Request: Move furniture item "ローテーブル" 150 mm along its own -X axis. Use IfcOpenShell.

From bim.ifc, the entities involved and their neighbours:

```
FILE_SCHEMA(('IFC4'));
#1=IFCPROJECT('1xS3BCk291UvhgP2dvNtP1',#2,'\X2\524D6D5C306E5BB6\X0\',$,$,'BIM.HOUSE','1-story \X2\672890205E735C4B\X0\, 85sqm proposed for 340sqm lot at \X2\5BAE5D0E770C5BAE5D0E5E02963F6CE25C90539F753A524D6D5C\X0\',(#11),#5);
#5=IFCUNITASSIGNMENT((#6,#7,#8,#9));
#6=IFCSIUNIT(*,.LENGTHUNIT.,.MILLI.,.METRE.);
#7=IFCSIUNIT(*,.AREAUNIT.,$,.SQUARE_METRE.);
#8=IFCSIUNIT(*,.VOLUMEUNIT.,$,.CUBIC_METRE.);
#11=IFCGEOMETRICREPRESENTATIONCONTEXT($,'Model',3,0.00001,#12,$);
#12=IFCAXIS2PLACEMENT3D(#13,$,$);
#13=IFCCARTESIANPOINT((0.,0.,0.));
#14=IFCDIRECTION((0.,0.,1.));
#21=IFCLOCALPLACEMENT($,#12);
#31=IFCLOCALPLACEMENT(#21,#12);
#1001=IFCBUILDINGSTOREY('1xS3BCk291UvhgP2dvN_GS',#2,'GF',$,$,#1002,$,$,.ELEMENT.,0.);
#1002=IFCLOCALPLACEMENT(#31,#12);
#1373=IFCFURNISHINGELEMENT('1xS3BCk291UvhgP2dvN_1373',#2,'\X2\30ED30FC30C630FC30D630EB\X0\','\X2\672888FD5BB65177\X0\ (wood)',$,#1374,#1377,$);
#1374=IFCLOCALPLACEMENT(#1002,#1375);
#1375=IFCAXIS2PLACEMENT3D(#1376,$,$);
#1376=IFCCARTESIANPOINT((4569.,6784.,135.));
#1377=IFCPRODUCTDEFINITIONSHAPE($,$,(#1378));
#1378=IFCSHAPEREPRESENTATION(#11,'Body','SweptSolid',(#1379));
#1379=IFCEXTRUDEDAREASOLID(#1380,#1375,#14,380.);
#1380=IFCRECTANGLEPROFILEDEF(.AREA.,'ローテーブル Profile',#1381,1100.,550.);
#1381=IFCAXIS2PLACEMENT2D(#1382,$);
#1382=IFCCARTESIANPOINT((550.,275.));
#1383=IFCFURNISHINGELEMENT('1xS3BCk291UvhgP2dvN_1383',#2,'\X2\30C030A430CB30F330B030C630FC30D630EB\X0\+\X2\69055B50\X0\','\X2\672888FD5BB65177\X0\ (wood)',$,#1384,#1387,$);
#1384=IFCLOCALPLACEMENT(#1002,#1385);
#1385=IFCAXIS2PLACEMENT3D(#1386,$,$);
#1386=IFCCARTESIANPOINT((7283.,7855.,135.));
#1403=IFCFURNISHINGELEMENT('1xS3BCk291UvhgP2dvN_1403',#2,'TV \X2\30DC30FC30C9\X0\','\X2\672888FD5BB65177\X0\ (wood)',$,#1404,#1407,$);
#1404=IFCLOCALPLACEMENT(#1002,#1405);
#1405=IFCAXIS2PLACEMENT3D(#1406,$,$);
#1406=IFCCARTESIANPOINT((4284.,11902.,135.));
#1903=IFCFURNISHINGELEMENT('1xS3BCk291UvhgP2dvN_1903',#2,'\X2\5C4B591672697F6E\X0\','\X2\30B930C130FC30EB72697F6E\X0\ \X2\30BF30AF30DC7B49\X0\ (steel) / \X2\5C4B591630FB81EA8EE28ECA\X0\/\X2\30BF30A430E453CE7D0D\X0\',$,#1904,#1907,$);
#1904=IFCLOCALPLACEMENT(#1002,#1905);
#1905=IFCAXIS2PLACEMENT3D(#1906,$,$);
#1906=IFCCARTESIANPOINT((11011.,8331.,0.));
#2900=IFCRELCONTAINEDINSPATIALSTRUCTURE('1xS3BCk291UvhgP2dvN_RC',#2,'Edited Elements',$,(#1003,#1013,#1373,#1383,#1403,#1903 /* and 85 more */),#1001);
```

```python
import ifcopenshell
import ifcopenshell.api.geometry
import ifcopenshell.util.placement
import ifcopenshell.util.unit

model = ifcopenshell.open("bim.ifc")
unit_scale = ifcopenshell.util.unit.calculate_unit_scale(model)

item = model.by_guid("1xS3BCk291UvhgP2dvN_1373")
matrix = ifcopenshell.util.placement.get_local_placement(item.ObjectPlacement)
matrix[:3, 3] -= matrix[:3, 0] * 0.15 / unit_scale
ifcopenshell.api.geometry.edit_object_placement(model, product=item, matrix=matrix, is_si=False)

print(ifcopenshell.util.placement.get_local_placement(item.ObjectPlacement).round(3) + 0.0)

model.write("bim_edited.ifc")
```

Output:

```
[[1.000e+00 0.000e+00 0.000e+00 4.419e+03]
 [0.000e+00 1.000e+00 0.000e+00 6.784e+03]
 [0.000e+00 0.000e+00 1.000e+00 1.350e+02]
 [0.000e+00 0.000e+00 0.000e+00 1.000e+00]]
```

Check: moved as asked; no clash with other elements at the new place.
